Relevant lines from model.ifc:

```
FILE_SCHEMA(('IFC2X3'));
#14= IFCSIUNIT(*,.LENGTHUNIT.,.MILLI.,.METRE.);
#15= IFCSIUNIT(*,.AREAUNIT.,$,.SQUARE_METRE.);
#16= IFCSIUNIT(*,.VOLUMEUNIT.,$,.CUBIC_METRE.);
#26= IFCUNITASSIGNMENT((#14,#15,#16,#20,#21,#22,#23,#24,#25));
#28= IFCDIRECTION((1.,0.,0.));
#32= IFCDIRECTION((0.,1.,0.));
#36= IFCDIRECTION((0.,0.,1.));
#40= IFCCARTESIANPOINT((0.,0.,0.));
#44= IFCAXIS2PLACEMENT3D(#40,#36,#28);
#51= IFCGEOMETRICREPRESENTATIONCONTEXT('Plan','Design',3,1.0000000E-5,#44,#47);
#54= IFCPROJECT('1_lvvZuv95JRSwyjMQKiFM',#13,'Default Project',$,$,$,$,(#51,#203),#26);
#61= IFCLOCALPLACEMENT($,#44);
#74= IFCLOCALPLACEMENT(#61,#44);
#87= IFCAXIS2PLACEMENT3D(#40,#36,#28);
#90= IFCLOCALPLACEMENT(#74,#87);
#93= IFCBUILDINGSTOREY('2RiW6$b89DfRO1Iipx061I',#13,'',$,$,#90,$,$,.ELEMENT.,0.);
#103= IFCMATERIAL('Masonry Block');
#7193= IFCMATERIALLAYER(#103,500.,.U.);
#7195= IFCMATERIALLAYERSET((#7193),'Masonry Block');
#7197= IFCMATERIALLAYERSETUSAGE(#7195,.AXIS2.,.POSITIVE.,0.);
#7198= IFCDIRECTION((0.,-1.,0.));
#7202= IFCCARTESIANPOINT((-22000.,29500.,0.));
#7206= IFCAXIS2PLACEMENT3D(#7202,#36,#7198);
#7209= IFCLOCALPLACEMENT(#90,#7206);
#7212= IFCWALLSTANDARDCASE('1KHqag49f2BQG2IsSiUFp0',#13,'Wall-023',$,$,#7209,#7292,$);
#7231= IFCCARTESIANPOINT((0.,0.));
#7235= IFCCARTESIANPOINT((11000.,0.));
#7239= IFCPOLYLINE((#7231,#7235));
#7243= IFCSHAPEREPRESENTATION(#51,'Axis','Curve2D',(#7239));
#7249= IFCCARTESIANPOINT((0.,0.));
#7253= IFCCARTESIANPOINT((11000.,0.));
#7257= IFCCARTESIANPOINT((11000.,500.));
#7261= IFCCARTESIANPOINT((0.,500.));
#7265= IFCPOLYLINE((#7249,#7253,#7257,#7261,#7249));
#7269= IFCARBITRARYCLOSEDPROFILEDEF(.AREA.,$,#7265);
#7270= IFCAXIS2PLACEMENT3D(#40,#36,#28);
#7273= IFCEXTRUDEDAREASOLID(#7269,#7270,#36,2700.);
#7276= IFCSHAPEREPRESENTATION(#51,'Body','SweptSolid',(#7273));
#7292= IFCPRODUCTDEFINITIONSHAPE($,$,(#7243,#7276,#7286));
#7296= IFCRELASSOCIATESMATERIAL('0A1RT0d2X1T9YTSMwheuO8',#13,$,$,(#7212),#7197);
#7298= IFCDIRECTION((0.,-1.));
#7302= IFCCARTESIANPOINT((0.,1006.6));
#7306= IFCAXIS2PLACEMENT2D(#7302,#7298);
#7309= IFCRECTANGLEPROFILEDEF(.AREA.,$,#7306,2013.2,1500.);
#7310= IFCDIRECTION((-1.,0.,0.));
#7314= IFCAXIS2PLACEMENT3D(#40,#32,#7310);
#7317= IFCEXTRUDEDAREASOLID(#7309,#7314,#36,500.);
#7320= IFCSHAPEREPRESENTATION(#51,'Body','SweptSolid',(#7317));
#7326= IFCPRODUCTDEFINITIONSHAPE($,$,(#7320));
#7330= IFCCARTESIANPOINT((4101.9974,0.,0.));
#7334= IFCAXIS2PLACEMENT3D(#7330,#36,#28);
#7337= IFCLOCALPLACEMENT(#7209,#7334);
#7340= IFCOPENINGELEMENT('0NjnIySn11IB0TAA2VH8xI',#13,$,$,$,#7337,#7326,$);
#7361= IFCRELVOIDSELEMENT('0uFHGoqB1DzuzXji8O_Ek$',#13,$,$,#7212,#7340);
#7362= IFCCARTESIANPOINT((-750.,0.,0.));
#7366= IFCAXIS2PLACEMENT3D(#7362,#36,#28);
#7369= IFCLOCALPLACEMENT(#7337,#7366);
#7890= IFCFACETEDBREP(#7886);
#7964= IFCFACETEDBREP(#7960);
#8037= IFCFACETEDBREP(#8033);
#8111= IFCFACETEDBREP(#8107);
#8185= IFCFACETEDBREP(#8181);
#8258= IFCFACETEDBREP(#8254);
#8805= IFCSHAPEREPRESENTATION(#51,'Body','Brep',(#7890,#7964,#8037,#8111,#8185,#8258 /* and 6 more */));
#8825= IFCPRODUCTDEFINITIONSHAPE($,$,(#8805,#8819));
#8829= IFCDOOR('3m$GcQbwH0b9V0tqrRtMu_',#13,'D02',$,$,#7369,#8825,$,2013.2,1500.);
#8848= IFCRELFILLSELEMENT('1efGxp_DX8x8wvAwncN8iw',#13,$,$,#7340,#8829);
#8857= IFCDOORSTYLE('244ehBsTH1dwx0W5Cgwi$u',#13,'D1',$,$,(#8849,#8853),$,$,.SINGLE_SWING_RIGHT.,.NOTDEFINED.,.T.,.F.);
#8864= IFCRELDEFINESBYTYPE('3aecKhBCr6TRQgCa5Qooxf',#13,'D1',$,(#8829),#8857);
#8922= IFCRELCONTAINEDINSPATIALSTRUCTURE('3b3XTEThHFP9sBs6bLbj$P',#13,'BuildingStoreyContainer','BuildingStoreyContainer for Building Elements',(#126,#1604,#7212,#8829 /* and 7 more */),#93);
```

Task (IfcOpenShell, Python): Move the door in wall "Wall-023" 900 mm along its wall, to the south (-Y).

```python
import ifcopenshell
import ifcopenshell.api.geometry
import ifcopenshell.util.placement

model = ifcopenshell.open("model.ifc")

door = model.by_guid("3m$GcQbwH0b9V0tqrRtMu_")
opening = door.FillsVoids[0].RelatingOpeningElement
wall = opening.VoidsElements[0].RelatingBuildingElement

wall_matrix = ifcopenshell.util.placement.get_local_placement(wall.ObjectPlacement)
shift = wall_matrix[:3, 0] * 900.0
before = ifcopenshell.util.placement.get_local_placement(door.ObjectPlacement)[:3, 3].copy()

# The door is placed relative to its opening, so it follows when the opening moves.
matrix = ifcopenshell.util.placement.get_local_placement(opening.ObjectPlacement)
matrix[:3, 3] += shift
ifcopenshell.api.geometry.edit_object_placement(
    model, product=opening, matrix=matrix, is_si=False, should_transform_children=True
)

after = ifcopenshell.util.placement.get_local_placement(door.ObjectPlacement)[:3, 3]
print("door moved by", (after - before).round(3) + 0.0)

model.write("model_rev.ifc")
```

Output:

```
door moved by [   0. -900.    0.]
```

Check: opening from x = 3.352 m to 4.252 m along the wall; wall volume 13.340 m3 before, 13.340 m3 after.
